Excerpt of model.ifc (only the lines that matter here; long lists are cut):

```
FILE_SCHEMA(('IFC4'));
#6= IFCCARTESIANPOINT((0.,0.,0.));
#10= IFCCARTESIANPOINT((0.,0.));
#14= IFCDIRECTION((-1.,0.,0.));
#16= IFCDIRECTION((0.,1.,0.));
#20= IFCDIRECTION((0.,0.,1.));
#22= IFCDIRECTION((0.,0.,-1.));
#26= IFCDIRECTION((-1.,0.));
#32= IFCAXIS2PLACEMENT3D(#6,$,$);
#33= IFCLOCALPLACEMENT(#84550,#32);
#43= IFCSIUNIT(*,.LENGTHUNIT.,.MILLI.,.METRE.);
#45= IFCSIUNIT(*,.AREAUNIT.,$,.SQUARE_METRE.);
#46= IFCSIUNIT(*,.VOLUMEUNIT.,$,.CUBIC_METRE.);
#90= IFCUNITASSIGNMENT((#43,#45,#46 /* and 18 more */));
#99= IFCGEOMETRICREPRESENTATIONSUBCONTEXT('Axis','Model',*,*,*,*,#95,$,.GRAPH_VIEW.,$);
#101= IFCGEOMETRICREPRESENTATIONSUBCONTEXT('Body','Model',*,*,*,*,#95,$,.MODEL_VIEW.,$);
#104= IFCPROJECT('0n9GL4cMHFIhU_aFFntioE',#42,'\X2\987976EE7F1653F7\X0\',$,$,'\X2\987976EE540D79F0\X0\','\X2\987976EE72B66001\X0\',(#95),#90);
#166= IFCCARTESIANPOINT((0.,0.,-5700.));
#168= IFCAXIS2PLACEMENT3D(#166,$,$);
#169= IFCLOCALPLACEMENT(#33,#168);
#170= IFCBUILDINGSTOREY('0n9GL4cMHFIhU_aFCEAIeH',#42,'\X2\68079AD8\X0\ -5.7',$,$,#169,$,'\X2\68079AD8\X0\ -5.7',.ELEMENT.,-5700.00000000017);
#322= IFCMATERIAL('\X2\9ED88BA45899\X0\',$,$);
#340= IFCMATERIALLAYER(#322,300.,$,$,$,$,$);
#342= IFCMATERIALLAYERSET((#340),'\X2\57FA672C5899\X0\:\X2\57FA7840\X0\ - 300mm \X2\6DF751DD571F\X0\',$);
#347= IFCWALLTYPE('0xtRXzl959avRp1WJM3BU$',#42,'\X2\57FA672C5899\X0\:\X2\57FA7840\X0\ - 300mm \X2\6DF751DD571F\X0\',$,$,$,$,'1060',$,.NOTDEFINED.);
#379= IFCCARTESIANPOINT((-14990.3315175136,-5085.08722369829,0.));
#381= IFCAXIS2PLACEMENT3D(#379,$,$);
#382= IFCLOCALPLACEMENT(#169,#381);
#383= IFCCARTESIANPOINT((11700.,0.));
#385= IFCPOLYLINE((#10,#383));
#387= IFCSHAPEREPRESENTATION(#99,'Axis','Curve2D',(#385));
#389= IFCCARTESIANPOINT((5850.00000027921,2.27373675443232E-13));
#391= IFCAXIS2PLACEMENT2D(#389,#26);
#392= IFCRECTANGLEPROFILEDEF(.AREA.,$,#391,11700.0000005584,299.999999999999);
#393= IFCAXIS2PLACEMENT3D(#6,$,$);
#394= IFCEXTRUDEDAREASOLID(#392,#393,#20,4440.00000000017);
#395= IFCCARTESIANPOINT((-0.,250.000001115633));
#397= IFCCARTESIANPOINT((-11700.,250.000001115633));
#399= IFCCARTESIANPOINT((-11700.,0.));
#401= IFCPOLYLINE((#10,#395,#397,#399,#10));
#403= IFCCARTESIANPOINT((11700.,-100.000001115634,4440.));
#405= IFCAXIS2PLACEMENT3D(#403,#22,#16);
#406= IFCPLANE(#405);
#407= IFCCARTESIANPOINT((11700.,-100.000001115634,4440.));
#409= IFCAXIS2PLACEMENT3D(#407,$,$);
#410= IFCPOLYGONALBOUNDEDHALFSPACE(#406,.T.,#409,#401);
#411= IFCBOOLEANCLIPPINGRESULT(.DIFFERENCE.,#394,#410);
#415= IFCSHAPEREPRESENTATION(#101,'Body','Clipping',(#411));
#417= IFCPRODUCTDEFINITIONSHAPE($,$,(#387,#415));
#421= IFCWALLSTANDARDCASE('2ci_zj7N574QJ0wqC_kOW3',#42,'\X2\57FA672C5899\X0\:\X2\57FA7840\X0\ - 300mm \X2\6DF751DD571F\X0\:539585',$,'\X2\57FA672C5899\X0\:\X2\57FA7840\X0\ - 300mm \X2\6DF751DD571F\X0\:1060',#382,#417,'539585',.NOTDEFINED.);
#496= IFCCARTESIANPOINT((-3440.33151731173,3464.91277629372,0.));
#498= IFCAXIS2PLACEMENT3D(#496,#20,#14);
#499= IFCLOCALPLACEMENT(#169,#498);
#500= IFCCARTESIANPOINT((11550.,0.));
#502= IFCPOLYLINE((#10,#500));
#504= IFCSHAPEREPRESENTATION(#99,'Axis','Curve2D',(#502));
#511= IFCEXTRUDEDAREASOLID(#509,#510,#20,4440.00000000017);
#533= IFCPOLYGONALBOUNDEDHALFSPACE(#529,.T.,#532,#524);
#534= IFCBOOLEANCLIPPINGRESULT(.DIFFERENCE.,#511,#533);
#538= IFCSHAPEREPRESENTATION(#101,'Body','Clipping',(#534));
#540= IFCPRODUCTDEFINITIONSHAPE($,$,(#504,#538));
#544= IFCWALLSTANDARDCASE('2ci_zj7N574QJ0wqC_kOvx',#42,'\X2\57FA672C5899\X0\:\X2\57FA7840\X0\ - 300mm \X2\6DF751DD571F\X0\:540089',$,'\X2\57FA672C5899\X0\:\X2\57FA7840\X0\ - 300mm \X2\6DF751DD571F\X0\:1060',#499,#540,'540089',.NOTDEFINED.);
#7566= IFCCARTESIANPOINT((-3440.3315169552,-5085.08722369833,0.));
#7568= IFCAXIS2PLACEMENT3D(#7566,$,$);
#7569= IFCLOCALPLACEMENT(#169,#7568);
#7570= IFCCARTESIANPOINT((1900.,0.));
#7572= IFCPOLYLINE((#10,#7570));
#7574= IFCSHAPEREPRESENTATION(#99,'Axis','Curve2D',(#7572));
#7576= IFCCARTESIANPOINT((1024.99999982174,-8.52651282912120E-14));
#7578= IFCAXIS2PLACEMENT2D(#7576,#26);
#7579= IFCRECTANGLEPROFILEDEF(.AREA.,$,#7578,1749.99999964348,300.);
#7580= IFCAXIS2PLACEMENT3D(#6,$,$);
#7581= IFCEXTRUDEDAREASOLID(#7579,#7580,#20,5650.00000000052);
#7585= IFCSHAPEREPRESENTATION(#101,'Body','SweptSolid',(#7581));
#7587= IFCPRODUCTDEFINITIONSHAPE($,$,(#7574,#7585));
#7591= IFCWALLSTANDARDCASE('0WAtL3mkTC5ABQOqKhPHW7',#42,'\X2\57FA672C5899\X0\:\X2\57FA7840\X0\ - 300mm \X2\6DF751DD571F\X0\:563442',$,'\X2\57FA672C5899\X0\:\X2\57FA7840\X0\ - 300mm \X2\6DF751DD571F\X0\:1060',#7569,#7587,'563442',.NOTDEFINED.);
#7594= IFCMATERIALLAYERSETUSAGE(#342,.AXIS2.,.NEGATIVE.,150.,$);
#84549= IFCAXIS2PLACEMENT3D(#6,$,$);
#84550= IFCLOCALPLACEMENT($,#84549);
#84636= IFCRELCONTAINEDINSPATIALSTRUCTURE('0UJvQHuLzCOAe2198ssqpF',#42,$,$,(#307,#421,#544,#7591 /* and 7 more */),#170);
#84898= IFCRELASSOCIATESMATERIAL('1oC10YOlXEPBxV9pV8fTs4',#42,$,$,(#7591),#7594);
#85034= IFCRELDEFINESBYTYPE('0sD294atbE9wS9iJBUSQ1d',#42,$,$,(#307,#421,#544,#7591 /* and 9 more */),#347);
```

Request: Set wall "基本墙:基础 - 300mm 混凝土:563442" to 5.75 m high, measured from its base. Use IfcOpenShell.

```python
import ifcopenshell
import ifcopenshell.geom
import ifcopenshell.util.representation
import ifcopenshell.util.shape

model = ifcopenshell.open("model.ifc")
settings = ifcopenshell.geom.settings()


def volume(element):
    """Net volume in cubic metres, openings subtracted."""
    shape = ifcopenshell.geom.create_shape(settings, element)
    return ifcopenshell.util.shape.get_volume(shape.geometry)


wall = model.by_id(7591)
before = volume(wall)

body = ifcopenshell.util.representation.get_representation(wall, "Model", "Body")
solid = body.Items[0]
old_height = solid.Depth
solid.Depth = 5750.0
after = volume(wall)

print(f"height {old_height:g} -> {solid.Depth:g}, volume {before:.3f} -> {after:.3f} m3")

model.write("model_rev.ifc")
```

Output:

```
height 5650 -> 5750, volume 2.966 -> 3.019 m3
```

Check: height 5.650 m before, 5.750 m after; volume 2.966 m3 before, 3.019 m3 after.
